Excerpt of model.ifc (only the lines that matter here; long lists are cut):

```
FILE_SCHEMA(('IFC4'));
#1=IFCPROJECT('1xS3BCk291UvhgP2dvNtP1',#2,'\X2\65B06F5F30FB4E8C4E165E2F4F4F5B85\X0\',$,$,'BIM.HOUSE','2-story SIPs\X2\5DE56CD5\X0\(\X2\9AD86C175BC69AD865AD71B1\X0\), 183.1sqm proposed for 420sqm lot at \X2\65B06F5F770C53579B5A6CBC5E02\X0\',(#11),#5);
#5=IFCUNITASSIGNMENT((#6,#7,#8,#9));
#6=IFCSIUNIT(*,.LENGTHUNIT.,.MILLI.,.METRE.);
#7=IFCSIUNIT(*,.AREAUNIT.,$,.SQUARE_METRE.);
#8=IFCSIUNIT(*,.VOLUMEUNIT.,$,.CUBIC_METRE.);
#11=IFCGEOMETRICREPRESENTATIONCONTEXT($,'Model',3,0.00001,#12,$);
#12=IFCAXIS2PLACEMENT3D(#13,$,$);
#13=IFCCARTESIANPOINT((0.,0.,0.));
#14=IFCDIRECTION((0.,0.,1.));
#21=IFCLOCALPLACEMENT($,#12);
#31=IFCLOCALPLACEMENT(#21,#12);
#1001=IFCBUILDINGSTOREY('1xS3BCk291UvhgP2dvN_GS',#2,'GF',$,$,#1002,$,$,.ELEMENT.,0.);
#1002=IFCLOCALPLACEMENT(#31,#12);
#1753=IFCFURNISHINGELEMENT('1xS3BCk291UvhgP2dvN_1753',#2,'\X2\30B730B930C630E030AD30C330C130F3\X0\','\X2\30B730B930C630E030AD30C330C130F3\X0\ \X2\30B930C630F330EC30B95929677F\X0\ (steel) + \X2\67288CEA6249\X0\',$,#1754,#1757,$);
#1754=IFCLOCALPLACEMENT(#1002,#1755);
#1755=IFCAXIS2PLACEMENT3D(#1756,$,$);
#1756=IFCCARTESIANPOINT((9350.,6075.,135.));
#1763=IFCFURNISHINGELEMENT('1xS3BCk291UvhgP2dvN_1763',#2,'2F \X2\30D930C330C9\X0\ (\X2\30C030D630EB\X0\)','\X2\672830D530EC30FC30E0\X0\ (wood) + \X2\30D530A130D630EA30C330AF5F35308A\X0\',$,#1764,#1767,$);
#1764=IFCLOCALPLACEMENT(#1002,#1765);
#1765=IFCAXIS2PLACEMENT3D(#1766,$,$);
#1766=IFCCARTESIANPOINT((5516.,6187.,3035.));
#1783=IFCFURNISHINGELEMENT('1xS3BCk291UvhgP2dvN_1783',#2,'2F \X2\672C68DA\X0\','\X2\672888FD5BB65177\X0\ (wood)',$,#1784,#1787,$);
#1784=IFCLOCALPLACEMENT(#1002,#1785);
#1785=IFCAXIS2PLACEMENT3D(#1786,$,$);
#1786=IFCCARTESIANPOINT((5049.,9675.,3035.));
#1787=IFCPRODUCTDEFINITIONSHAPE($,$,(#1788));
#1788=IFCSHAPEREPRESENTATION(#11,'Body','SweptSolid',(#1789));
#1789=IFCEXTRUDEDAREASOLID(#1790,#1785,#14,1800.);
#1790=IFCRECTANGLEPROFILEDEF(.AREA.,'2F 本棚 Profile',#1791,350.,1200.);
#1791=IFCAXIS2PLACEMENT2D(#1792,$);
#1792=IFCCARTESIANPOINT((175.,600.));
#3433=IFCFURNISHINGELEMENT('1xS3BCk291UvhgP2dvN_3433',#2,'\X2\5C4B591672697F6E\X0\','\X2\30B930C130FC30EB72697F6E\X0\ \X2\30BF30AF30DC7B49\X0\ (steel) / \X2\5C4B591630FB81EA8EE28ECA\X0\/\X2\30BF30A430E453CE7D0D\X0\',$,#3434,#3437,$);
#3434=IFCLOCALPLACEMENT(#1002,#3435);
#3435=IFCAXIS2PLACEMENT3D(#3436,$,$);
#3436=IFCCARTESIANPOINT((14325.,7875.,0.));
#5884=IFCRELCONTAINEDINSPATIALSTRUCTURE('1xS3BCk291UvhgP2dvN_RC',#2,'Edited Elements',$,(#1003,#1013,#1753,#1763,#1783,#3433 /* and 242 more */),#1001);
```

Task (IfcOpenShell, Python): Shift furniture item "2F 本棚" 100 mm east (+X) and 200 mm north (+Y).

```python
import ifcopenshell
import ifcopenshell.api.geometry
import ifcopenshell.util.placement

model = ifcopenshell.open("model.ifc")

item = model.by_id(1783)
matrix = ifcopenshell.util.placement.get_local_placement(item.ObjectPlacement)
matrix[0, 3] += 100.0
matrix[1, 3] += 200.0
ifcopenshell.api.geometry.edit_object_placement(model, product=item, matrix=matrix, is_si=False)

print(ifcopenshell.util.placement.get_local_placement(item.ObjectPlacement).round(3) + 0.0)

model.write("model_rev.ifc")
```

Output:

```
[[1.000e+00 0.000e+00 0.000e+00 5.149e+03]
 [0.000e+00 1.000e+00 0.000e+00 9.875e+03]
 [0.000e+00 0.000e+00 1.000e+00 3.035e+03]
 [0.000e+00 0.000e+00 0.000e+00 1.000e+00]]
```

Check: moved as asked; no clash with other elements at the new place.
